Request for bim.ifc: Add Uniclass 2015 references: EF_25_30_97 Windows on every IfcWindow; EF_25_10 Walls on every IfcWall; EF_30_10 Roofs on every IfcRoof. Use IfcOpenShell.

First a look at what the model holds.

```python
import ifcopenshell

model = ifcopenshell.open("bim.ifc")
print(model.schema)
print("classifications:", [c.Name for c in model.by_type("IfcClassification")])
for ifc_class in ("IfcDoor", "IfcRoof", "IfcStair", "IfcWall", "IfcWindow"):
    print(ifc_class, len(model.by_type(ifc_class)))
```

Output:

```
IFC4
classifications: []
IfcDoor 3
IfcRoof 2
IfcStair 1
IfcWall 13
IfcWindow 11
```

```python
import ifcopenshell
import ifcopenshell.api.classification

model = ifcopenshell.open("bim.ifc")

system = ifcopenshell.api.classification.add_classification(model, classification="Uniclass 2015")

codes = {
    "IfcWindow": ("EF_25_30_97", "Windows"),
    "IfcWall": ("EF_25_10", "Walls"),
    "IfcRoof": ("EF_30_10", "Roofs"),
}
for ifc_class, (code, name) in codes.items():
    products = model.by_type(ifc_class)
    ifcopenshell.api.classification.add_reference(
        model, products=products, classification=system, identification=code, name=name
    )
    print(code, len(products))

model.write("bim_edited.ifc")
```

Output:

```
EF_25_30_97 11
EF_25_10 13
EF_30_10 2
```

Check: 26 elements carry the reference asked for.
